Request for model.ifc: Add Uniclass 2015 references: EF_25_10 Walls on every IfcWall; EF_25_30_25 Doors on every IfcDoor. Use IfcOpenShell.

First a look at what the model holds.

```python
import ifcopenshell

model = ifcopenshell.open("model.ifc")
print(model.schema)
print("classifications:", [c.Name for c in model.by_type("IfcClassification")])
for ifc_class in ("IfcDoor", "IfcRoof", "IfcStair", "IfcWall", "IfcWindow"):
    print(ifc_class, len(model.by_type(ifc_class)))
```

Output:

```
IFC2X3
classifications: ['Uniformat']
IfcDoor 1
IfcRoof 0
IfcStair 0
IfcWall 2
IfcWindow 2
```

```python
import ifcopenshell
import ifcopenshell.api.classification

model = ifcopenshell.open("model.ifc")

# IFC2X3 requires Source and Edition and has no link from the project to the system.
system = model.create_entity("IfcClassification", Source="NBS", Edition="2015", Name="Uniclass 2015")

codes = {
    "IfcWall": ("EF_25_10", "Walls"),
    "IfcDoor": ("EF_25_30_25", "Doors"),
}
for ifc_class, (code, name) in codes.items():
    products = model.by_type(ifc_class)
    ifcopenshell.api.classification.add_reference(
        model, products=products, classification=system, identification=code, name=name
    )
    print(code, len(products))

model.write("model_rev.ifc")
```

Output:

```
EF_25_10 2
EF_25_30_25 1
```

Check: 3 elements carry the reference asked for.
